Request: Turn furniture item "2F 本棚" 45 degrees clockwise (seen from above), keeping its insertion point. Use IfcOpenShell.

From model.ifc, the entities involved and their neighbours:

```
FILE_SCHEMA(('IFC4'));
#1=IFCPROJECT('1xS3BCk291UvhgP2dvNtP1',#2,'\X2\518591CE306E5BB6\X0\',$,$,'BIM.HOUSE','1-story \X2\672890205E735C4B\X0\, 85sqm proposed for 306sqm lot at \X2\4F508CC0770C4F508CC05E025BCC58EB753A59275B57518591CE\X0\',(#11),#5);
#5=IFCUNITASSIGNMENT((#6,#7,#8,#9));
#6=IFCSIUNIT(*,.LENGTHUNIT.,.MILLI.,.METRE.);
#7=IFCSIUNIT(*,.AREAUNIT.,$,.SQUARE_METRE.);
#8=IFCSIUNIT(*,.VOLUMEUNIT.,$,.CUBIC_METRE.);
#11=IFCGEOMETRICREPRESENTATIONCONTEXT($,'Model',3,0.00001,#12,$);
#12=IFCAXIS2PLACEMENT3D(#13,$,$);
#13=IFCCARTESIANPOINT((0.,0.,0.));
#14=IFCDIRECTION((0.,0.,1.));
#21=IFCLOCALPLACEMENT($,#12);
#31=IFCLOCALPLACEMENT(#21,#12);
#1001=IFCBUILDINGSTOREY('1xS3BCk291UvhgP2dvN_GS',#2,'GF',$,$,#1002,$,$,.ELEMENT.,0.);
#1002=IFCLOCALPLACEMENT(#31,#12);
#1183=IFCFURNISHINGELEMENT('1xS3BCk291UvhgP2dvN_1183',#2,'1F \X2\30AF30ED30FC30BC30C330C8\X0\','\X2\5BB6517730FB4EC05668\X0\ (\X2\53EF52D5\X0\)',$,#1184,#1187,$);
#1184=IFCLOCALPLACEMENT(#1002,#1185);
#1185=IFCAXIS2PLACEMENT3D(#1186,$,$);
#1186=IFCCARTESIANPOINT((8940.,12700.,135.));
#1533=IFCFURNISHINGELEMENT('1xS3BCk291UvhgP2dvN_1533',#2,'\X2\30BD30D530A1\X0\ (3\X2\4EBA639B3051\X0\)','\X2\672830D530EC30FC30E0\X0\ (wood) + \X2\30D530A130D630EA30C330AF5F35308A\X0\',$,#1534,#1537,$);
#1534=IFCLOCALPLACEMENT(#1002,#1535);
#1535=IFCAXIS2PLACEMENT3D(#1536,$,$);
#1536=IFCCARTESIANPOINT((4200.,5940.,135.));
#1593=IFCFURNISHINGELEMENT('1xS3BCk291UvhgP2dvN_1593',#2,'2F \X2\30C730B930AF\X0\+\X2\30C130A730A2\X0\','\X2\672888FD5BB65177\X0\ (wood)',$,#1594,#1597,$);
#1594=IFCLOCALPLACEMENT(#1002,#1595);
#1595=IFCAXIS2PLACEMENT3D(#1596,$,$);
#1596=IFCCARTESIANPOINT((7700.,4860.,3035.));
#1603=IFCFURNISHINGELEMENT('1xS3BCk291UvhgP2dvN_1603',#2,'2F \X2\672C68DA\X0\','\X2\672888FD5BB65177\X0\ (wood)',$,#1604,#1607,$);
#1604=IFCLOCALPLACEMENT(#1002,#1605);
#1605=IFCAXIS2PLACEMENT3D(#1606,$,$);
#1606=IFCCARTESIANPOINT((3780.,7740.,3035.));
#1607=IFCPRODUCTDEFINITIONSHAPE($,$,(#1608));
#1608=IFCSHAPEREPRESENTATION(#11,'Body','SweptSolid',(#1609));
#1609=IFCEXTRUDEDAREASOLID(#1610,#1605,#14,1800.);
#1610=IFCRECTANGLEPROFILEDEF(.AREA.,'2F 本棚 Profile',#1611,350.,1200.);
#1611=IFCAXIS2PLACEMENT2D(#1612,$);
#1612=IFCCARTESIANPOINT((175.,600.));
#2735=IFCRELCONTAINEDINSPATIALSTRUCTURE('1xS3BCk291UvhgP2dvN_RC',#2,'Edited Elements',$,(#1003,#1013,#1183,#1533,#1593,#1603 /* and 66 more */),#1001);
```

```python
import ifcopenshell
import ifcopenshell.api.geometry
import ifcopenshell.util.placement

model = ifcopenshell.open("model.ifc")

item = model.by_guid("1xS3BCk291UvhgP2dvN_1603")
matrix = ifcopenshell.util.placement.get_local_placement(item.ObjectPlacement)
matrix = matrix @ ifcopenshell.util.placement.rotation(-45, "Z")
ifcopenshell.api.geometry.edit_object_placement(model, product=item, matrix=matrix, is_si=False)

print(ifcopenshell.util.placement.get_local_placement(item.ObjectPlacement).round(3) + 0.0)

model.write("model-out.ifc")
```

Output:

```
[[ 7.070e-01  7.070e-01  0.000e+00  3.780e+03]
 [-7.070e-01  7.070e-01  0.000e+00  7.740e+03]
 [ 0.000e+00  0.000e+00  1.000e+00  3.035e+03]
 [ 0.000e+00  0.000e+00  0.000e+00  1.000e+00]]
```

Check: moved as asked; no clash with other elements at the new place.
